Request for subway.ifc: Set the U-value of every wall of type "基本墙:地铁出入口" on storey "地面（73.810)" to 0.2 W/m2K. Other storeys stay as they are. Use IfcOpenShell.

First a look at what the model holds.

```python
import ifcopenshell
import ifcopenshell.util.element

model = ifcopenshell.open("subway.ifc")
print(model.schema)
storey = next(s for s in model.by_type("IfcBuildingStorey") if s.Name == "地面（73.810)")
walls = [e for e in ifcopenshell.util.element.get_decomposition(storey) if e.is_a("IfcWall")]
seen = {}
for e in walls:
    element_type = ifcopenshell.util.element.get_type(e)
    key = (element_type.Name if element_type != e and element_type else None, ifcopenshell.util.element.get_pset(e, "Pset_WallCommon", "ThermalTransmittance"))
    seen[key] = seen.get(key, 0) + 1
for (name, value), count in sorted(seen.items(), key=str):
    print(count, "x", name, "|", value)
```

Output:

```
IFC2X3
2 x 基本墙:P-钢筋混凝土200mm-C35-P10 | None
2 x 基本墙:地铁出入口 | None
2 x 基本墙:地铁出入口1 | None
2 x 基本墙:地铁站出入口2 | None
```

```python
import ifcopenshell
import ifcopenshell.api.pset
import ifcopenshell.util.element

model = ifcopenshell.open("subway.ifc")

storey = next(s for s in model.by_type("IfcBuildingStorey") if s.Name == "地面（73.810)")
walls = [e for e in ifcopenshell.util.element.get_decomposition(storey) if e.is_a("IfcWall")]

count = 0
for e in walls:
    element_type = ifcopenshell.util.element.get_type(e)
    if element_type in (None, e) or element_type.Name != "基本墙:地铁出入口":
        continue
    # add_pset returns the element's existing set when there is one.
    pset = ifcopenshell.api.pset.add_pset(model, product=e, name="Pset_WallCommon")
    ifcopenshell.api.pset.edit_pset(model, pset=pset, properties={"ThermalTransmittance": 0.2})
    count += 1

print(count, "walls updated")

model.write("subway_v2.ifc")
```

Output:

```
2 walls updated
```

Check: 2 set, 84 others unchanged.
